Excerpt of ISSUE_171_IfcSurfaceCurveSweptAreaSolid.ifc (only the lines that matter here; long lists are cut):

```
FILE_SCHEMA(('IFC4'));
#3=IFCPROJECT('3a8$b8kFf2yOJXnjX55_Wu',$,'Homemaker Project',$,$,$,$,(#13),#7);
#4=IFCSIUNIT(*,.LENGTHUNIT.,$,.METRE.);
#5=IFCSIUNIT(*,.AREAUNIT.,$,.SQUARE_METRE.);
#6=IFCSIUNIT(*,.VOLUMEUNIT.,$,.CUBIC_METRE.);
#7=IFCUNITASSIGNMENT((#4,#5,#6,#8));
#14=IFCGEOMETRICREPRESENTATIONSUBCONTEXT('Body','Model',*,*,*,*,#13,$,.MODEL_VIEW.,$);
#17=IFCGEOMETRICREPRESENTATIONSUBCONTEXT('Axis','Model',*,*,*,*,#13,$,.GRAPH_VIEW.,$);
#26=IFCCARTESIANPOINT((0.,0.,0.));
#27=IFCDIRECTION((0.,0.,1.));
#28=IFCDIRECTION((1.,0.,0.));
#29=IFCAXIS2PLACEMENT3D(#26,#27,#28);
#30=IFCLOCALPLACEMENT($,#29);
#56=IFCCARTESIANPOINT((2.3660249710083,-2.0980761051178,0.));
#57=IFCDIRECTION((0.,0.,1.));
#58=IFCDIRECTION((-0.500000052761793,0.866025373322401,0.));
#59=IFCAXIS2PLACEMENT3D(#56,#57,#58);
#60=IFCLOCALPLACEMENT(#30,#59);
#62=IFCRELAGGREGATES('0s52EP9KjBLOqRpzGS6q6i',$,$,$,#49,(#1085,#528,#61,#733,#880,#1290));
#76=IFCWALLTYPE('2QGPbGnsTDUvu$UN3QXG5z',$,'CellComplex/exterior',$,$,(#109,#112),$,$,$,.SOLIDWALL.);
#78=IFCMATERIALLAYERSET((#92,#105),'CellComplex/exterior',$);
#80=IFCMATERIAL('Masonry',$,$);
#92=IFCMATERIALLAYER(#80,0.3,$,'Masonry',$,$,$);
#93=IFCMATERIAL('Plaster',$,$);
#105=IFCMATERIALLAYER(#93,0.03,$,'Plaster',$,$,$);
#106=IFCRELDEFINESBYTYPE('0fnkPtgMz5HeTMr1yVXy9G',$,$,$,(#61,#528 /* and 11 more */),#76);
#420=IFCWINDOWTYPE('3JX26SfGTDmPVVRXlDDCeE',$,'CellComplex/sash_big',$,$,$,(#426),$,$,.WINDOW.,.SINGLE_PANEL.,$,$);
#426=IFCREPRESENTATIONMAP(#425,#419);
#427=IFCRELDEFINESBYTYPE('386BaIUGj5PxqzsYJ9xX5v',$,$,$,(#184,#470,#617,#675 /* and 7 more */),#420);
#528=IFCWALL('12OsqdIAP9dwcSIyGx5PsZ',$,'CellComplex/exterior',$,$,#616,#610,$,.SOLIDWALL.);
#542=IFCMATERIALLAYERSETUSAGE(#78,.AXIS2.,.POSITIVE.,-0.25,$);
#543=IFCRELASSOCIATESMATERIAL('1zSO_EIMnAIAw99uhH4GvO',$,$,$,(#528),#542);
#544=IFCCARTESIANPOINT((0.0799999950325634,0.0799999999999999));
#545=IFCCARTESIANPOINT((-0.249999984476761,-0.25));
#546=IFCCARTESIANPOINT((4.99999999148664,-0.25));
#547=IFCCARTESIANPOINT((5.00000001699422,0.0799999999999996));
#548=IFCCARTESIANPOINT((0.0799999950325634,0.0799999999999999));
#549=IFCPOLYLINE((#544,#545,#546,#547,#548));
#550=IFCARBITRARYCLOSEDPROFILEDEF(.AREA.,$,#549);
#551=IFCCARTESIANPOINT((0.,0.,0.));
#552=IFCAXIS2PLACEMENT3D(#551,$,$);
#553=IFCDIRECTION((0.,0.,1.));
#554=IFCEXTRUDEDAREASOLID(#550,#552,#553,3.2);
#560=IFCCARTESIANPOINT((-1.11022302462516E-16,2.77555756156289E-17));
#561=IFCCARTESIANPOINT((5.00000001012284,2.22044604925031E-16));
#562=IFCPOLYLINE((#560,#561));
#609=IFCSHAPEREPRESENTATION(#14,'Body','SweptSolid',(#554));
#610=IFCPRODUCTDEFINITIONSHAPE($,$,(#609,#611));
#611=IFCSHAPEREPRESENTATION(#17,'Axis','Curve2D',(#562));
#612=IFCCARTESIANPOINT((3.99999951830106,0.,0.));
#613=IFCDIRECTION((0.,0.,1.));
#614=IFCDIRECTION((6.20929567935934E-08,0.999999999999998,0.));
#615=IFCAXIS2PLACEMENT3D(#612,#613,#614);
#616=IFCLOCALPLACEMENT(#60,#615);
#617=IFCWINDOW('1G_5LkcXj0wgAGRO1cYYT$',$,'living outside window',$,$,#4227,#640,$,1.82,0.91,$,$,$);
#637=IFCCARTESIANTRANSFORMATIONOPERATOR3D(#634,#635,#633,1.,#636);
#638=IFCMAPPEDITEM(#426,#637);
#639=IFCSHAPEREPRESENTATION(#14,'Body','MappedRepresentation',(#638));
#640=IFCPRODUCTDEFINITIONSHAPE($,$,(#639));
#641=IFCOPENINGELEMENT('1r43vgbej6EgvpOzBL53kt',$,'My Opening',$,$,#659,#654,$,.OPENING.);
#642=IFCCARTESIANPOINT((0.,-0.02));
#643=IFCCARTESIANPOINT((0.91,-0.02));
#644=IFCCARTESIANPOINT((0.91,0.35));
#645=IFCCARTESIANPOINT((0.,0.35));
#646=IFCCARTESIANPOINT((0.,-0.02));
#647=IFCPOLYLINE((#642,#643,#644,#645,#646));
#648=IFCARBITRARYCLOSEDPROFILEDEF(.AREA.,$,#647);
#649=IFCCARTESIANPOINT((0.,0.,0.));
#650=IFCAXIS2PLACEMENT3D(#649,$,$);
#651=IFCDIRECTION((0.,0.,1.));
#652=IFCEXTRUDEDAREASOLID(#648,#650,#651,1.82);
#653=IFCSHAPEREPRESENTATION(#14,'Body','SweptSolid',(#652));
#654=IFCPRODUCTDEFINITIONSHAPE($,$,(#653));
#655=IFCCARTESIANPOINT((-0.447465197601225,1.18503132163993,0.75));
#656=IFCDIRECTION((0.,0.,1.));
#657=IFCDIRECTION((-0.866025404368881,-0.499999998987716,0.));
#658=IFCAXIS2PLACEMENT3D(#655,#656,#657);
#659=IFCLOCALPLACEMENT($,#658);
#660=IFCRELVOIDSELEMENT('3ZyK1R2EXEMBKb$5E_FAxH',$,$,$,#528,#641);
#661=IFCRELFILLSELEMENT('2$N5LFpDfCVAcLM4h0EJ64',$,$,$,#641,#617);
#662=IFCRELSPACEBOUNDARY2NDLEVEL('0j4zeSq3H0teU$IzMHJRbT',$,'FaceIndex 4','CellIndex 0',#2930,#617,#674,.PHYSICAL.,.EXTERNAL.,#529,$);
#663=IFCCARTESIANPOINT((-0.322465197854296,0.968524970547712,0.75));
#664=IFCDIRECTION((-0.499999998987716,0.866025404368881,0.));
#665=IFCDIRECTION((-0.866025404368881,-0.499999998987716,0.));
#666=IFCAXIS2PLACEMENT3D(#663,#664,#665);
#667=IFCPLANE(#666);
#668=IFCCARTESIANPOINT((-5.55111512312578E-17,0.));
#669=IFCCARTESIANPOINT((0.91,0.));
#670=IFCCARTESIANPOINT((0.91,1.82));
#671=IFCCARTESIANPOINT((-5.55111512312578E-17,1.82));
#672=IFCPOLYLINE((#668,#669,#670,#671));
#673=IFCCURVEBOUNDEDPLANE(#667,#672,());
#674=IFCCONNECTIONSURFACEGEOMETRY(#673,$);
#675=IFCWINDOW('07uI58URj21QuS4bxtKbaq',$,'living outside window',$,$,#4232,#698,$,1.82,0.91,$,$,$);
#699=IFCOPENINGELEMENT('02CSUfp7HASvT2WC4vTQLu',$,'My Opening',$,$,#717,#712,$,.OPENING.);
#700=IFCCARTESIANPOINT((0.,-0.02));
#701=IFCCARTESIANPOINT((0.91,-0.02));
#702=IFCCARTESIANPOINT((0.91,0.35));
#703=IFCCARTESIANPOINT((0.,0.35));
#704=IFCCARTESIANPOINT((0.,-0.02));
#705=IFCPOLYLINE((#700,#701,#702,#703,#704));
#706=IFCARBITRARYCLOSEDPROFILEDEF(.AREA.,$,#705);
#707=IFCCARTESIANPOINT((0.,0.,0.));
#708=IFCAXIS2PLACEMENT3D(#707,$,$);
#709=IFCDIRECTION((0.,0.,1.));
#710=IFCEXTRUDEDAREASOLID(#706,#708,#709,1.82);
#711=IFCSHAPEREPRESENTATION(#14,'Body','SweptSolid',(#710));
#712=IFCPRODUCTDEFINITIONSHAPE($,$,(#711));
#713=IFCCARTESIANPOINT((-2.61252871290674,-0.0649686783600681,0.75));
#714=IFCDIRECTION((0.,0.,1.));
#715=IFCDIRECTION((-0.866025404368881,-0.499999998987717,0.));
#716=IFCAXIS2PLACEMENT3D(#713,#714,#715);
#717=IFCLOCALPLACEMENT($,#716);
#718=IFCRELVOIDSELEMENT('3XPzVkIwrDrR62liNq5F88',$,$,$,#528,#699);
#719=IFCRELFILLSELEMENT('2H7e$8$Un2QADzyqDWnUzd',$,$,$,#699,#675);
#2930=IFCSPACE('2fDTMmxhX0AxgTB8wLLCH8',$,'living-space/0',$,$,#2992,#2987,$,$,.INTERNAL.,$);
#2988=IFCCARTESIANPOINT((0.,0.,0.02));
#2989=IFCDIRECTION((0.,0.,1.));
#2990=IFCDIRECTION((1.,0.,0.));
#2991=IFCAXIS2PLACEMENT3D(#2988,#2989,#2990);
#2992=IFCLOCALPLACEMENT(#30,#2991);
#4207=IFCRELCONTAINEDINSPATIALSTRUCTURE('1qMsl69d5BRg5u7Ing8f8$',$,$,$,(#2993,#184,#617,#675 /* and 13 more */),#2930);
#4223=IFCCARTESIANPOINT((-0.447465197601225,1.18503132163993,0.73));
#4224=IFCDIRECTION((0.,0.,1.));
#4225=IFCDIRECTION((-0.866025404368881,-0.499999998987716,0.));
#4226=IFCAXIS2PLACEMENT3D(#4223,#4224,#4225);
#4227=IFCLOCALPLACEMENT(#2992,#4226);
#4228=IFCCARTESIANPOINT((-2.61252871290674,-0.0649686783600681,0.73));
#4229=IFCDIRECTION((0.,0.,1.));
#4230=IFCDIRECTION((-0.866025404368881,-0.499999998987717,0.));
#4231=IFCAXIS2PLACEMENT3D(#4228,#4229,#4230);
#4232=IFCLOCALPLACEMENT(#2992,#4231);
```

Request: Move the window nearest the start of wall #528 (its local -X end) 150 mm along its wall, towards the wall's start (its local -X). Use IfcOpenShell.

```python
import numpy as np
import ifcopenshell
import ifcopenshell.api.geometry
import ifcopenshell.util.placement
import ifcopenshell.util.unit

model = ifcopenshell.open("ISSUE_171_IfcSurfaceCurveSweptAreaSolid.ifc")
unit_scale = ifcopenshell.util.unit.calculate_unit_scale(model)

window = model.by_id(617)
opening = window.FillsVoids[0].RelatingOpeningElement
wall = opening.VoidsElements[0].RelatingBuildingElement

wall_matrix = ifcopenshell.util.placement.get_local_placement(wall.ObjectPlacement)
shift = wall_matrix[:3, 0] * -0.15 / unit_scale
before = ifcopenshell.util.placement.get_local_placement(window.ObjectPlacement)[:3, 3].copy()

# The window is not placed relative to its opening, so move both.
for product in (opening, window):
    matrix = ifcopenshell.util.placement.get_local_placement(product.ObjectPlacement)
    matrix[:3, 3] += shift
    ifcopenshell.api.geometry.edit_object_placement(model, product=product, matrix=matrix, is_si=False)

# Space boundary surfaces are stored in each space's coordinates; move them too.
for rel in window.ProvidesBoundaries:
    if not rel.ConnectionGeometry:
        continue
    surface = rel.ConnectionGeometry.SurfaceOnRelatingElement.BasisSurface
    space_matrix = ifcopenshell.util.placement.get_local_placement(rel.RelatingSpace.ObjectPlacement)
    point = np.array(surface.Position.Location.Coordinates) + space_matrix[:3, :3].T @ shift
    surface.Position = model.createIfcAxis2Placement3D(
        model.createIfcCartesianPoint(point.tolist()), surface.Position.Axis, surface.Position.RefDirection
    )

after = ifcopenshell.util.placement.get_local_placement(window.ObjectPlacement)[:3, 3]
print("window moved by", (after - before).round(3) + 0.0)

model.write("ISSUE_171_IfcSurfaceCurveSweptAreaSolid_edited.ifc")
```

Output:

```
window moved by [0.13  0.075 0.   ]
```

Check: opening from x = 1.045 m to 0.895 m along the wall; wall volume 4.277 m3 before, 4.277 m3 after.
